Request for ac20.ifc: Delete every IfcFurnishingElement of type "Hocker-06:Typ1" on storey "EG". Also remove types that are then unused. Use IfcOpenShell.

First a look at what the model holds.

```python
import ifcopenshell
import ifcopenshell.util.element

model = ifcopenshell.open("ac20.ifc")
print(model.schema)
storey = next(s for s in model.by_type("IfcBuildingStorey") if s.Name == "EG")
furniture = [e for e in ifcopenshell.util.element.get_decomposition(storey) if e.is_a("IfcFurnishingElement")]
seen = {}
for e in furniture:
    element_type = ifcopenshell.util.element.get_type(e)
    name = element_type.Name if element_type not in (None, e) else None
    seen[name] = seen.get(name, 0) + 1
for name, count in sorted(seen.items(), key=str):
    print(count, "x", name)
```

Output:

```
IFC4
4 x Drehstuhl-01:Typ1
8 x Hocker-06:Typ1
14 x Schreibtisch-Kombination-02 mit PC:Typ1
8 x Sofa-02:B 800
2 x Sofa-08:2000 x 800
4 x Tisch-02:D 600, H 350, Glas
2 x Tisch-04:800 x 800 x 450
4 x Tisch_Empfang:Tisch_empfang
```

```python
import ifcopenshell
import ifcopenshell.api.root
import ifcopenshell.util.element

model = ifcopenshell.open("ac20.ifc")

storey = next(s for s in model.by_type("IfcBuildingStorey") if s.Name == "EG")
furniture = [e for e in ifcopenshell.util.element.get_decomposition(storey) if e.is_a("IfcFurnishingElement")]
targets = [e for e in furniture if (t := ifcopenshell.util.element.get_type(e)) not in (None, e) and t.Name == "Hocker-06:Typ1"]
types = {ifcopenshell.util.element.get_type(e) for e in targets} - {None, *targets}

for e in targets:
    ifcopenshell.api.root.remove_product(model, product=e)
print(len(targets), "removed")

unused = [t for t in types if not ifcopenshell.util.element.get_types(t)]
for t in unused:
    ifcopenshell.api.root.remove_product(model, product=t)
print(len(unused), "unused types removed")

model.write("ac20-out.ifc")
```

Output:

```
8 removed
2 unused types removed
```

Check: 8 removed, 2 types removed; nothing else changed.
